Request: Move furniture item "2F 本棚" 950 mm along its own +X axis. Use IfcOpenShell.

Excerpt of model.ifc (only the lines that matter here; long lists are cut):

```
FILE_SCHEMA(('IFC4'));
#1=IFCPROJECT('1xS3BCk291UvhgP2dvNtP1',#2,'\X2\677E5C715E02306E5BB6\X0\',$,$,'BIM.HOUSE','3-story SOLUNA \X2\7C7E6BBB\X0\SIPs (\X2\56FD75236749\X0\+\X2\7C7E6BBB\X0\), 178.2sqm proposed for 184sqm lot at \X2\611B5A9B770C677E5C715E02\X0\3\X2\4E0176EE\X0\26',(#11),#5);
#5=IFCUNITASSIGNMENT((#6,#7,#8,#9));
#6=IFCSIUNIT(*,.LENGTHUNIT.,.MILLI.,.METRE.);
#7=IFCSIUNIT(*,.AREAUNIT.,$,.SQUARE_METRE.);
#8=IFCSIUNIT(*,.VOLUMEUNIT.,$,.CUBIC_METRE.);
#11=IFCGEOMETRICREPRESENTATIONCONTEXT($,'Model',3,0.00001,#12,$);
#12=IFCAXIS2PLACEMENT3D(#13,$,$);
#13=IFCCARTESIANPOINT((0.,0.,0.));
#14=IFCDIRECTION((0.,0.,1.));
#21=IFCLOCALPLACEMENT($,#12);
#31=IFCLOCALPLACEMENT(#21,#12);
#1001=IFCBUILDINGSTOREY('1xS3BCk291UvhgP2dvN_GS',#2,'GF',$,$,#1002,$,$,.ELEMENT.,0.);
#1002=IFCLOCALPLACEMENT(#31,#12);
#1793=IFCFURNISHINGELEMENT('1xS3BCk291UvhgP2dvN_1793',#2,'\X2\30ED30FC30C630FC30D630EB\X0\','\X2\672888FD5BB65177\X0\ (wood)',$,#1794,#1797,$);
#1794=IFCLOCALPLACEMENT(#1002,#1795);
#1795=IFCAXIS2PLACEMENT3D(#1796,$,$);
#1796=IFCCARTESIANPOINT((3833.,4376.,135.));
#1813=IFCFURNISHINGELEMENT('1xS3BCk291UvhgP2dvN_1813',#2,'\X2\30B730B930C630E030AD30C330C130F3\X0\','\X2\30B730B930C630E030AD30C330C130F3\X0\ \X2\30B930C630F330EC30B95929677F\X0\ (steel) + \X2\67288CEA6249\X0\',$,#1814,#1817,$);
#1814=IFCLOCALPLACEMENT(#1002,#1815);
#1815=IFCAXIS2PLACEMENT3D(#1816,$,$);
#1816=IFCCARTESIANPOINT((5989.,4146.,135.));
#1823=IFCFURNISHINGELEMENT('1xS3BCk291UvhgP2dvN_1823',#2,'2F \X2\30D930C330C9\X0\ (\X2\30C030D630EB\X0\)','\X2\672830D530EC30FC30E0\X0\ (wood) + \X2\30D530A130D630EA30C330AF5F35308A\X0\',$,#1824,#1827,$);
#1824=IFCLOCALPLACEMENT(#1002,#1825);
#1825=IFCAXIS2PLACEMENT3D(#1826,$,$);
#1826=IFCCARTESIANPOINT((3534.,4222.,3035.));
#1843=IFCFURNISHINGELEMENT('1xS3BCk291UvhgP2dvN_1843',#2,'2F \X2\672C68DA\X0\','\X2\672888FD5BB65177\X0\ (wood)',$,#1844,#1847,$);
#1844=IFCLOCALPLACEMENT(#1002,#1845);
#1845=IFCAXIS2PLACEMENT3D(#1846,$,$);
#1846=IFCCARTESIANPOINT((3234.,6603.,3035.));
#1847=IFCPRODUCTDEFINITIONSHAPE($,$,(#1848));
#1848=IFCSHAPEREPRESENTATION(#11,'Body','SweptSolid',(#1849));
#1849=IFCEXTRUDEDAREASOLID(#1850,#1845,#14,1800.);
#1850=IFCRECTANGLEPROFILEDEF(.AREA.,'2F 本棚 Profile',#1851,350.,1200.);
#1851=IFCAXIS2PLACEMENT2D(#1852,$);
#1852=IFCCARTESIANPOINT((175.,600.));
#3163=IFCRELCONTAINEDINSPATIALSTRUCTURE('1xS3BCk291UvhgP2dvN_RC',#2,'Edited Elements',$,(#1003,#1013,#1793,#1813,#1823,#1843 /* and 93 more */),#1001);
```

```python
import ifcopenshell
import ifcopenshell.api.geometry
import ifcopenshell.util.placement

model = ifcopenshell.open("model.ifc")

item = model.by_guid("1xS3BCk291UvhgP2dvN_1843")
matrix = ifcopenshell.util.placement.get_local_placement(item.ObjectPlacement)
matrix[:3, 3] += matrix[:3, 0] * 950.0
ifcopenshell.api.geometry.edit_object_placement(model, product=item, matrix=matrix, is_si=False)

print(ifcopenshell.util.placement.get_local_placement(item.ObjectPlacement).round(3) + 0.0)

model.write("model-out.ifc")
```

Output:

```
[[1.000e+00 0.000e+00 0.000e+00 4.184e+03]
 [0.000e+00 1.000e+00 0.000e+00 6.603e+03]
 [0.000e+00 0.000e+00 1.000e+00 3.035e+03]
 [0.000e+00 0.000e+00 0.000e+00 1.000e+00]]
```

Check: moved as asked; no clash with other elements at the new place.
